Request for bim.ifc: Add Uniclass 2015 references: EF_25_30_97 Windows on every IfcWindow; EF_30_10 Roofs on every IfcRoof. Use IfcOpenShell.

First a look at what the model holds.

```python
import ifcopenshell

model = ifcopenshell.open("bim.ifc")
print(model.schema)
print("classifications:", [c.Name for c in model.by_type("IfcClassification")])
for ifc_class in ("IfcDoor", "IfcRoof", "IfcStair", "IfcWall", "IfcWindow"):
    print(ifc_class, len(model.by_type(ifc_class)))
```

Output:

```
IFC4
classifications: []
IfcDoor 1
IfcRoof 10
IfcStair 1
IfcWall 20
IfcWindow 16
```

```python
import ifcopenshell
import ifcopenshell.api.classification

model = ifcopenshell.open("bim.ifc")

system = ifcopenshell.api.classification.add_classification(model, classification="Uniclass 2015")

codes = {
    "IfcWindow": ("EF_25_30_97", "Windows"),
    "IfcRoof": ("EF_30_10", "Roofs"),
}
for ifc_class, (code, name) in codes.items():
    products = model.by_type(ifc_class)
    ifcopenshell.api.classification.add_reference(
        model, products=products, classification=system, identification=code, name=name
    )
    print(code, len(products))

model.write("bim-out.ifc")
```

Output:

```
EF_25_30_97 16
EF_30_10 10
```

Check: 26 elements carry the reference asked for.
